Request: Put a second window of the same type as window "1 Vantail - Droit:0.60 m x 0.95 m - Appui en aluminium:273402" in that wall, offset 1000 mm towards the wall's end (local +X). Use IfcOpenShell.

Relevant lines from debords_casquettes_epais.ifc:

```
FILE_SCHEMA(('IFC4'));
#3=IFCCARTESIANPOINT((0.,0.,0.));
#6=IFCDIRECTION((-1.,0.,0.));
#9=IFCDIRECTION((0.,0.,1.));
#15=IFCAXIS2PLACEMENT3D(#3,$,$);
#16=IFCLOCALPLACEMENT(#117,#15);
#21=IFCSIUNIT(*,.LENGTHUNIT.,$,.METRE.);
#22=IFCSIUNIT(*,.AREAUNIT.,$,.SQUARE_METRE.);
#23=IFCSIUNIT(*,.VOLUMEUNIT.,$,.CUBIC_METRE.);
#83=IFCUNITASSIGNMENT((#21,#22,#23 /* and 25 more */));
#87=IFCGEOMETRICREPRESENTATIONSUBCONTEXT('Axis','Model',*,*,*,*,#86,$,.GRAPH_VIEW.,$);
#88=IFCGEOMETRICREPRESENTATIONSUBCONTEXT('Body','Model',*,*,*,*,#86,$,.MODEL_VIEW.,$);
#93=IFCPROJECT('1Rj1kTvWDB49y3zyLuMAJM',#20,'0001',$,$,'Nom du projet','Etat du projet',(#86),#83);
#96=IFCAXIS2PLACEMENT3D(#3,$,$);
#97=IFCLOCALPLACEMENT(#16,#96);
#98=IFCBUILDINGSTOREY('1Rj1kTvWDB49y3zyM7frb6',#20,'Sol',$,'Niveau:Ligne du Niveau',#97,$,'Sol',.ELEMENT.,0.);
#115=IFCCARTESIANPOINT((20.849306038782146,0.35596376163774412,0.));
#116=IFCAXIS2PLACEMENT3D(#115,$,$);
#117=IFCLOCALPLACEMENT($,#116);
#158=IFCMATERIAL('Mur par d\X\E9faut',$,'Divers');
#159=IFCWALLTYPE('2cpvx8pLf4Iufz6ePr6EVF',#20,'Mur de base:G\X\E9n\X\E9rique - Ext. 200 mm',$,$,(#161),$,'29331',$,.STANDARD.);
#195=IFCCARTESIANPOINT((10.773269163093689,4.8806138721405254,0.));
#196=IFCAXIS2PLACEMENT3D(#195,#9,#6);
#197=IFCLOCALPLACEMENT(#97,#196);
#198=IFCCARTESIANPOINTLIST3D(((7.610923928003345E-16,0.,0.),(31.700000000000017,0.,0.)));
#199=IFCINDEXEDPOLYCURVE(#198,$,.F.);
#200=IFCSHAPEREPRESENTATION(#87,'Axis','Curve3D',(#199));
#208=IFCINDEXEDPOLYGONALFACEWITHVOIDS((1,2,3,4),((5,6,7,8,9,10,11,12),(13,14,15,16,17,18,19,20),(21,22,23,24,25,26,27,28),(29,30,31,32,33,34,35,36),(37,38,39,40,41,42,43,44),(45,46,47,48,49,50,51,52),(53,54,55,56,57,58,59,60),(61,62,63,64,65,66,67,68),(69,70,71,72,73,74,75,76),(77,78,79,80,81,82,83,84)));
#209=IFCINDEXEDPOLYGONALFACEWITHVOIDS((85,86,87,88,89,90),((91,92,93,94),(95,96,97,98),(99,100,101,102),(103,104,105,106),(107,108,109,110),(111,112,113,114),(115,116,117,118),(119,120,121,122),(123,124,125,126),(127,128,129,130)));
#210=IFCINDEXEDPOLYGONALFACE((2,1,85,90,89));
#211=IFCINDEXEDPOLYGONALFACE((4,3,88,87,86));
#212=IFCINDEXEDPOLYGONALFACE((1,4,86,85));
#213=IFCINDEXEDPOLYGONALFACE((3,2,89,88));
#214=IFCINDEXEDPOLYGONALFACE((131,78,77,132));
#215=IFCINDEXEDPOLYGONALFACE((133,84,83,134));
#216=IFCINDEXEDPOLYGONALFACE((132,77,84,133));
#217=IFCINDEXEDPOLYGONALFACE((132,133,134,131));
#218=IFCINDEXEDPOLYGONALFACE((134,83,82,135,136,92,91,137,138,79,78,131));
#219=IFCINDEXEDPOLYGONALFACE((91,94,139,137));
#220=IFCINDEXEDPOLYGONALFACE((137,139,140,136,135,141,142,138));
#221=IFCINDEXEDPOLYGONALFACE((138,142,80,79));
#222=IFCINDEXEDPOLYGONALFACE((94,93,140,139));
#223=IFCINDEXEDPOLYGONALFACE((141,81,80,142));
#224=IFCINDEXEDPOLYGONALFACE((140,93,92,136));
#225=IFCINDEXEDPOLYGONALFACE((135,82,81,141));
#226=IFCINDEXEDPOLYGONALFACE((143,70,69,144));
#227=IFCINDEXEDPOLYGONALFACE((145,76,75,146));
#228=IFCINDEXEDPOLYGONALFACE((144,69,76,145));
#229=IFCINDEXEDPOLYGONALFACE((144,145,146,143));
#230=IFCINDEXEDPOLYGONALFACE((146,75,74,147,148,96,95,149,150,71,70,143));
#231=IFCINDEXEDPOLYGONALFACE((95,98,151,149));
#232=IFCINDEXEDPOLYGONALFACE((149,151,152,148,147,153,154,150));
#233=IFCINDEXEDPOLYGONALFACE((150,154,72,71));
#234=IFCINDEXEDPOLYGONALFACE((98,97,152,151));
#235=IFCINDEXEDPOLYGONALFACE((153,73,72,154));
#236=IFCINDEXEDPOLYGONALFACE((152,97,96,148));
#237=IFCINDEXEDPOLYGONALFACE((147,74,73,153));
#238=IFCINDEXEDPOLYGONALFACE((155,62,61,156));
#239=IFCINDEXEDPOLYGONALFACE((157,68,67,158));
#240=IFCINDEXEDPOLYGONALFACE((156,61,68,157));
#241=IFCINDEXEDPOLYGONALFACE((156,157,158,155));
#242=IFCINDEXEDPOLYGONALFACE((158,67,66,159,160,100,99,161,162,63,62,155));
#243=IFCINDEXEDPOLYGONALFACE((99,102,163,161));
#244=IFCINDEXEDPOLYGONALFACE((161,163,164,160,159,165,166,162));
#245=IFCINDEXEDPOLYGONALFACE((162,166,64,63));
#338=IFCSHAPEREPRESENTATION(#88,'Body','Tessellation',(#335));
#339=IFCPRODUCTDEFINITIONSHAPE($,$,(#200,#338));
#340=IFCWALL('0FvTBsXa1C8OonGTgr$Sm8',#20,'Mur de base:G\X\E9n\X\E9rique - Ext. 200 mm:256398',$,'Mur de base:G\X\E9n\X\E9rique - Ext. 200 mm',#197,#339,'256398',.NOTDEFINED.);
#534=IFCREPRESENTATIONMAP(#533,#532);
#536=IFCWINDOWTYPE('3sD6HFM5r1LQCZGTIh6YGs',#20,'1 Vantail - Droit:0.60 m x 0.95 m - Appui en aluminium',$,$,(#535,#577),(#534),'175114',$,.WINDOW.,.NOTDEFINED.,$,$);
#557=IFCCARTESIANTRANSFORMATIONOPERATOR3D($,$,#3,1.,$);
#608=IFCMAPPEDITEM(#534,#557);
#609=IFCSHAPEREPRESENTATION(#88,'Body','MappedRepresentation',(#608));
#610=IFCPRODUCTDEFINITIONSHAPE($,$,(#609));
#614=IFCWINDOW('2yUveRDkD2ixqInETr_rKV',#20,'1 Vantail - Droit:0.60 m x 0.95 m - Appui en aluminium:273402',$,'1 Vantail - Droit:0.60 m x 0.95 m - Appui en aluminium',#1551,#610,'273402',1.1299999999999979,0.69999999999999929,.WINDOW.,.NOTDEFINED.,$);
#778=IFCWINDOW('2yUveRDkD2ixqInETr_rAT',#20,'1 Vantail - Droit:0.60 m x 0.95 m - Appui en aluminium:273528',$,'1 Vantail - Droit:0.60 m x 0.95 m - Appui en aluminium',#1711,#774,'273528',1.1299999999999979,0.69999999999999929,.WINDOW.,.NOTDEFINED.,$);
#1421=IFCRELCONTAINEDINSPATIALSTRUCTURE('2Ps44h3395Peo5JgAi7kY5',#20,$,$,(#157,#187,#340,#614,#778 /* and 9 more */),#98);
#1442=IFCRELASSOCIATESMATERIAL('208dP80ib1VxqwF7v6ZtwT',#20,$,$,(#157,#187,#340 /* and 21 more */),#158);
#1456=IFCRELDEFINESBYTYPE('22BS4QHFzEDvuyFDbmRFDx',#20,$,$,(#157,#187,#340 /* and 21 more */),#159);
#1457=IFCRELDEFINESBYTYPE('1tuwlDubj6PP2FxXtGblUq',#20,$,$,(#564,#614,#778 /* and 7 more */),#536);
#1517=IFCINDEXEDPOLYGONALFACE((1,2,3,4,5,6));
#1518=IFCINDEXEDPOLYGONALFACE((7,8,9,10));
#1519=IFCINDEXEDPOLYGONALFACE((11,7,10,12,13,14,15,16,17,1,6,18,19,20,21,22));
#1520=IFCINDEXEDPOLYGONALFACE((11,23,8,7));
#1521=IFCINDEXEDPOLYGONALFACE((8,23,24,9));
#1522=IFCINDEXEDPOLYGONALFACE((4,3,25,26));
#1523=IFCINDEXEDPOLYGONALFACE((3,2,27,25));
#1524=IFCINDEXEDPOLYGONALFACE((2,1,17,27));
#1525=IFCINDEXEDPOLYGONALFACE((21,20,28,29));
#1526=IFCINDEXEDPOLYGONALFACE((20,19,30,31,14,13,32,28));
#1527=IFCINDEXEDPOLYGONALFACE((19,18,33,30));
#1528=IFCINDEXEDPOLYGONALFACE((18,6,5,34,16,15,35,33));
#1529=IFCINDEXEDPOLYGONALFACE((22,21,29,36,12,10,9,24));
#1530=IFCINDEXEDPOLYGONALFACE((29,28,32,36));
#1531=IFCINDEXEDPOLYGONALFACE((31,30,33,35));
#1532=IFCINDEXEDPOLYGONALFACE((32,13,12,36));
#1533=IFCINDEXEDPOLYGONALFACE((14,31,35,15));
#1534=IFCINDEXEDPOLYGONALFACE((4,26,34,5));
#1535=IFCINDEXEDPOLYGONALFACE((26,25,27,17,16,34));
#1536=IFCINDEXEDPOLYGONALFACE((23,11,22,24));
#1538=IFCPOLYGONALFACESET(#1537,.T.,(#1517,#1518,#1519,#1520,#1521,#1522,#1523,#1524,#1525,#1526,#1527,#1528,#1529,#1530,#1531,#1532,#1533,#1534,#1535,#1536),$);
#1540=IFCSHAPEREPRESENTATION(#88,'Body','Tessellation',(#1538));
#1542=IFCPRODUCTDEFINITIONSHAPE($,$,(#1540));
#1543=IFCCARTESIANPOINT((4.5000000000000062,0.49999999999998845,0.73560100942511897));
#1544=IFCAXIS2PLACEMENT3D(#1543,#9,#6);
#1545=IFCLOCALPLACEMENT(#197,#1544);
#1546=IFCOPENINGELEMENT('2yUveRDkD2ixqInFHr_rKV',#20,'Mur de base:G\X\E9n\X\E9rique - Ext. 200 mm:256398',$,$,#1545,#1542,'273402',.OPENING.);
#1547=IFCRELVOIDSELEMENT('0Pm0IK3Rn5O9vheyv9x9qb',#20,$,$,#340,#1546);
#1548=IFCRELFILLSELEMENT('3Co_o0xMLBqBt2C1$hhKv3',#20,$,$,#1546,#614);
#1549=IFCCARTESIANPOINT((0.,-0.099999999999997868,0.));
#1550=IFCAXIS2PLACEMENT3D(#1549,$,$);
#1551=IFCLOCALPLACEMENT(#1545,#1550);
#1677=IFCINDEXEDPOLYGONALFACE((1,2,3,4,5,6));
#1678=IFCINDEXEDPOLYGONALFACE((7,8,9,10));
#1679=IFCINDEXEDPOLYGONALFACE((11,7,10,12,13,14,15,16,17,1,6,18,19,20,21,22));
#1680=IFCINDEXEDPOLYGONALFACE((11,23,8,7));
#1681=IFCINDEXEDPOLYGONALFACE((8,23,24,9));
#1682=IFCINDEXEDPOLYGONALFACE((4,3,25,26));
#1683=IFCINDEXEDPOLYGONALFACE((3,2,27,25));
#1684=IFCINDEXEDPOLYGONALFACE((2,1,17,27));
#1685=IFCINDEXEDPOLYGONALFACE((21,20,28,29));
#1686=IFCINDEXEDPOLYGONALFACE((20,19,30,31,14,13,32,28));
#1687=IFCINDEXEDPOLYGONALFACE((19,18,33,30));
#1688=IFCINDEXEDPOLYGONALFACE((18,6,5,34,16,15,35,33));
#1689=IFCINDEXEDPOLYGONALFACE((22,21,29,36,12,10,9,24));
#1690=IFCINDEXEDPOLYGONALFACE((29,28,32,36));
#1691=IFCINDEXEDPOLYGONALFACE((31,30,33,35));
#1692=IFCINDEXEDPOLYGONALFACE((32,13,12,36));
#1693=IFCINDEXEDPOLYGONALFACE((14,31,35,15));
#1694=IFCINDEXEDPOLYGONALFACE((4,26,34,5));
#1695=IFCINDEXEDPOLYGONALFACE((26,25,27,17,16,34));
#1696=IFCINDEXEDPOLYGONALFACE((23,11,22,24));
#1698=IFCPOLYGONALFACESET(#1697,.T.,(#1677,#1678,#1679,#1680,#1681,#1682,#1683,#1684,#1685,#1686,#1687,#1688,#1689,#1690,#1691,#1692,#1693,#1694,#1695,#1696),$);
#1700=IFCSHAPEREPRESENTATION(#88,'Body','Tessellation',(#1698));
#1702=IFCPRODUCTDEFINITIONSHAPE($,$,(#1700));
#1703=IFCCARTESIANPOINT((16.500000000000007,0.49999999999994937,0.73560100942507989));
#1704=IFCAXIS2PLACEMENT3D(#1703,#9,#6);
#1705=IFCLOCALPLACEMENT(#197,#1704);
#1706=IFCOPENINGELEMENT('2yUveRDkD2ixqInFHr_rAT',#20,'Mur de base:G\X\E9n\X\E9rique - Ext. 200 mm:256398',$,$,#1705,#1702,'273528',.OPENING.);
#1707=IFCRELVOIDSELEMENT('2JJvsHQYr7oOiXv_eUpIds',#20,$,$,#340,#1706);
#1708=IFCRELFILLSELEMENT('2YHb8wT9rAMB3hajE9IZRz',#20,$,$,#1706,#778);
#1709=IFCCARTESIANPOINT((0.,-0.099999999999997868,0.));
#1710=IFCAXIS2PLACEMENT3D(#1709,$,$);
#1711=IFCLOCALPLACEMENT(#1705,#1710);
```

```python
import ifcopenshell
import ifcopenshell.api.feature
import ifcopenshell.api.geometry
import ifcopenshell.api.root
import ifcopenshell.geom
import ifcopenshell.util.element
import ifcopenshell.util.placement
import ifcopenshell.util.shape

model = ifcopenshell.open("debords_casquettes_epais.ifc")
settings = ifcopenshell.geom.settings()


def volume(element):
    """Net volume in cubic metres, openings subtracted."""
    shape = ifcopenshell.geom.create_shape(settings, element)
    return ifcopenshell.util.shape.get_volume(shape.geometry)


def reuse_history(source, copy):
    """copy_class also copies each property set's owner history, people and application; keep the originals."""
    for rel in copy.IsDefinedBy:
        if rel.is_a("IfcRelDefinesByProperties") and (history := rel.RelatingPropertyDefinition.OwnerHistory):
            rel.RelatingPropertyDefinition.OwnerHistory = source.OwnerHistory
            ifcopenshell.util.element.remove_deep2(model, history)


window = model.by_guid("2yUveRDkD2ixqInETr_rKV")
opening = window.FillsVoids[0].RelatingOpeningElement
wall = opening.VoidsElements[0].RelatingBuildingElement
before = volume(wall)
shift = ifcopenshell.util.placement.get_local_placement(wall.ObjectPlacement)[:3, 0] * 1.0

# copy_class copies the void relationship, type, container and properties, but no geometry.
new_opening = ifcopenshell.api.root.copy_class(model, product=opening)
new_opening.Representation = ifcopenshell.util.element.copy_deep(
    model, opening.Representation, exclude=["IfcGeometricRepresentationContext", "IfcRepresentationMap"]
)
new_opening.Name = "Mur de base:Générique - Ext. 200 mm"
new_opening.Tag = None
new_window = ifcopenshell.api.root.copy_class(model, product=window)
new_window.Representation = ifcopenshell.util.element.copy_deep(
    model, window.Representation, exclude=["IfcGeometricRepresentationContext", "IfcRepresentationMap"]
)
new_window.Name = "1 Vantail - Droit:0.60 m x 0.95 m - Appui en aluminium"
new_window.Tag = None
reuse_history(window, new_window)
ifcopenshell.api.feature.add_filling(model, opening=new_opening, element=new_window)

for old, new in ((opening, new_opening), (window, new_window)):
    matrix = ifcopenshell.util.placement.get_local_placement(old.ObjectPlacement)
    matrix[:3, 3] += shift
    ifcopenshell.api.geometry.edit_object_placement(model, product=new, matrix=matrix, is_si=False)

after = volume(wall)

print(f"wall volume {before:.3f} -> {after:.3f} m3")

model.write("debords_casquettes_epais_v2.ifc")
```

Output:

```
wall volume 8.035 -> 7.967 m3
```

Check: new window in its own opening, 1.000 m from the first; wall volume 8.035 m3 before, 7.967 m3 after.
